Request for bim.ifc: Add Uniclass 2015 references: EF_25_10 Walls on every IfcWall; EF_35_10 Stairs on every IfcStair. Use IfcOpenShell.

First a look at what the model holds.

```python
import ifcopenshell

model = ifcopenshell.open("bim.ifc")
print(model.schema)
print("classifications:", [c.Name for c in model.by_type("IfcClassification")])
for ifc_class in ("IfcDoor", "IfcRoof", "IfcStair", "IfcWall", "IfcWindow"):
    print(ifc_class, len(model.by_type(ifc_class)))
```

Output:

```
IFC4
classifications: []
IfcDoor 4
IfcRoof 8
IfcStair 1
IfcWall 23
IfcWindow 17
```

```python
import ifcopenshell
import ifcopenshell.api.classification

model = ifcopenshell.open("bim.ifc")

system = ifcopenshell.api.classification.add_classification(model, classification="Uniclass 2015")

codes = {
    "IfcWall": ("EF_25_10", "Walls"),
    "IfcStair": ("EF_35_10", "Stairs"),
}
for ifc_class, (code, name) in codes.items():
    products = model.by_type(ifc_class)
    ifcopenshell.api.classification.add_reference(
        model, products=products, classification=system, identification=code, name=name
    )
    print(code, len(products))

model.write("bim_updated.ifc")
```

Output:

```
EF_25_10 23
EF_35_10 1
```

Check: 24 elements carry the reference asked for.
